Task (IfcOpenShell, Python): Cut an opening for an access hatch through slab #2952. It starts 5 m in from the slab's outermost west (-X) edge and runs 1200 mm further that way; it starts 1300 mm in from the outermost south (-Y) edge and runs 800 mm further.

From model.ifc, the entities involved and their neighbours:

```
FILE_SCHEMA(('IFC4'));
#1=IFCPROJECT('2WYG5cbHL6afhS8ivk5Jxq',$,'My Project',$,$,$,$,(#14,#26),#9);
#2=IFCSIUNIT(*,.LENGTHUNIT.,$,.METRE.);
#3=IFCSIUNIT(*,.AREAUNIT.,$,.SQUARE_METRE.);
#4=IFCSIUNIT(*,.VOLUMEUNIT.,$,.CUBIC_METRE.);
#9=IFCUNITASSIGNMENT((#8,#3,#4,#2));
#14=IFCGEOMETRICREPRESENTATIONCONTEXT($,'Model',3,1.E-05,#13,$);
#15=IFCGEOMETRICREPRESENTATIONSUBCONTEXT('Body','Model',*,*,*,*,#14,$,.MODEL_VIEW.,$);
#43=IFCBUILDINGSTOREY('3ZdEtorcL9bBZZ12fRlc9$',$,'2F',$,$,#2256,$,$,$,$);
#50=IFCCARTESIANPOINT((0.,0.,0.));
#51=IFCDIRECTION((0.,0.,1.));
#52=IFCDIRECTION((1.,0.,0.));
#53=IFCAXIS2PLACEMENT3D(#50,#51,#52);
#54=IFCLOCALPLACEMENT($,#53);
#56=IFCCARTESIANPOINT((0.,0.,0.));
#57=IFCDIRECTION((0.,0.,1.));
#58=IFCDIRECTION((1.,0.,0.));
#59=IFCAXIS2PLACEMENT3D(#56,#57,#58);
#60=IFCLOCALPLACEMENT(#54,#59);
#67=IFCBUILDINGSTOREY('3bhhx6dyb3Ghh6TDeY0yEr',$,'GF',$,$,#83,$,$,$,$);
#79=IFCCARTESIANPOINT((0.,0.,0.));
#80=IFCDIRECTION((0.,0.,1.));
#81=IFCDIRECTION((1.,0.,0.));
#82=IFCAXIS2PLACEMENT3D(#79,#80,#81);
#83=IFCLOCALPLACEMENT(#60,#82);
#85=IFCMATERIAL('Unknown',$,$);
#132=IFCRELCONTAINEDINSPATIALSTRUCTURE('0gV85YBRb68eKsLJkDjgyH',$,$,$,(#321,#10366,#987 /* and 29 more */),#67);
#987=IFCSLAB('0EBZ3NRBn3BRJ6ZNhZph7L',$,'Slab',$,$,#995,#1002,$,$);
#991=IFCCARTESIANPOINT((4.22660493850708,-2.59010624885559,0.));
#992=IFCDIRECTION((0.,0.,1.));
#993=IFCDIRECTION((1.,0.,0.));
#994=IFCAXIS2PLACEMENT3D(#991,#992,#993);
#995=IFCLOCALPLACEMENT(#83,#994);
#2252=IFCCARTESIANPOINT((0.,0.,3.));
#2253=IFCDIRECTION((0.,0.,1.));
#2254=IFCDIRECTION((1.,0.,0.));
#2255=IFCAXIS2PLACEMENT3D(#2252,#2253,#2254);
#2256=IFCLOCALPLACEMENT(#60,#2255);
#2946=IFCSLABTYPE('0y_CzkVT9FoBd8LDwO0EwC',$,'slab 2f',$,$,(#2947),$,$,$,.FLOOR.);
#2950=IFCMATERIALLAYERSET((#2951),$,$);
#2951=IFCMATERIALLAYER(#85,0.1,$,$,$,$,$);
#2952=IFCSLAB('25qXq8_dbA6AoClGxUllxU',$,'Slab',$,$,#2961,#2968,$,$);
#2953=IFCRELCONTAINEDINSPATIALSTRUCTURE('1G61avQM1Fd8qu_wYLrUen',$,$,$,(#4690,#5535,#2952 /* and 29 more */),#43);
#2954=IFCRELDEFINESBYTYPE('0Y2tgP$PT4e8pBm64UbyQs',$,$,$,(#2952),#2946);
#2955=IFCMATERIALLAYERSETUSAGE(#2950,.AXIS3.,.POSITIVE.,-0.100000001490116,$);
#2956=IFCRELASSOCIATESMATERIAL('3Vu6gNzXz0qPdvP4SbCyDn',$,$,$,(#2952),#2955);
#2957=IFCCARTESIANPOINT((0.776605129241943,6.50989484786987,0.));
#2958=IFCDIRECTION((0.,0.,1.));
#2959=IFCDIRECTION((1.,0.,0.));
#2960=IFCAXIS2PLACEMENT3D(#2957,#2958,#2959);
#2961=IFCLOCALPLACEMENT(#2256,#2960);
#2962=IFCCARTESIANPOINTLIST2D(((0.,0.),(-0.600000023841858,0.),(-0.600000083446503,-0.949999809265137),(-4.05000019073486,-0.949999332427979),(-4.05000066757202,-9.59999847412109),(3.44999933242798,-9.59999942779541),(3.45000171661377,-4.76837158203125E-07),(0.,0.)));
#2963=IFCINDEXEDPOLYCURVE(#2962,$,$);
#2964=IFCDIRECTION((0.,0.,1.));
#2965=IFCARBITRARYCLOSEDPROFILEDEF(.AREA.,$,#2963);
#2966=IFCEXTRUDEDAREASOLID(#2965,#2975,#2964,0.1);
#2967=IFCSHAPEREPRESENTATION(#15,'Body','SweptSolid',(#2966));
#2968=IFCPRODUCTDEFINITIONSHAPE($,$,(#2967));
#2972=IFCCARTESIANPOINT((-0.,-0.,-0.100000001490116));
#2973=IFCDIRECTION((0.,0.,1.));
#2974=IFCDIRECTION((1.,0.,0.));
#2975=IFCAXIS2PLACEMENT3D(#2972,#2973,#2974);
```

```python
import numpy as np
import ifcopenshell
import ifcopenshell.api.feature
import ifcopenshell.api.geometry
import ifcopenshell.api.root
import ifcopenshell.geom
import ifcopenshell.util.placement
import ifcopenshell.util.representation
import ifcopenshell.util.shape
import ifcopenshell.util.unit

model = ifcopenshell.open("model.ifc")
unit_scale = ifcopenshell.util.unit.calculate_unit_scale(model)
settings = ifcopenshell.geom.settings()


def volume(element):
    """Net volume in cubic metres, openings subtracted."""
    shape = ifcopenshell.geom.create_shape(settings, element)
    return ifcopenshell.util.shape.get_volume(shape.geometry)


slab = model.by_id(2952)
before = volume(slab)

# Extent in the slab's own axes, in metres. The edges named are its -X and -Y sides.
slab_shape = ifcopenshell.geom.create_shape(settings, slab)
vertices = ifcopenshell.util.shape.get_vertices(slab_shape.geometry)
x_min, y_min, bottom = vertices.min(axis=0)
top = vertices[:, 2].max()

opening = ifcopenshell.api.root.create_entity(model, ifc_class="IfcOpeningElement", name="Access hatch opening", predefined_type="OPENING")
context = ifcopenshell.util.representation.get_context(model, "Model", "Body", "MODEL_VIEW")
width, depth = 1.2, 0.8
outline = [(0.0, 0.0), (width, 0.0), (width, depth), (0.0, depth), (0.0, 0.0)]
# Overshoot both faces by 50 mm so the cut is clean.
shape = ifcopenshell.api.geometry.add_slab_representation(
    model, context=context, depth=top - bottom + 0.1, polyline=outline
)
ifcopenshell.api.geometry.assign_representation(model, product=opening, representation=shape)

matrix = ifcopenshell.util.placement.get_local_placement(slab.ObjectPlacement)
matrix[:, 3] = matrix @ np.append(np.array([x_min + 5, y_min + 1.3, bottom - 0.05]) / unit_scale, 1.0)
ifcopenshell.api.geometry.edit_object_placement(model, product=opening, matrix=matrix, is_si=False)
ifcopenshell.api.feature.add_feature(model, feature=opening, element=slab)

after = volume(slab)

print(f"slab volume {before:.3f} -> {after:.3f} m3")

model.write("model_edited.ifc")
```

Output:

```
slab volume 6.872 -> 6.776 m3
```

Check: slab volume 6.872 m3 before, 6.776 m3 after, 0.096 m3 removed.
